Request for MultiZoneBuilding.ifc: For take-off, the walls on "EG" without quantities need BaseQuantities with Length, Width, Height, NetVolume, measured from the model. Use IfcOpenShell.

First a look at what the model holds.

```python
import ifcopenshell
import ifcopenshell.util.element
import ifcopenshell.util.unit

model = ifcopenshell.open("MultiZoneBuilding.ifc")
print(model.schema)
for unit_type in ("LENGTHUNIT", "AREAUNIT", "VOLUMEUNIT"):
    print(unit_type, ifcopenshell.util.unit.calculate_unit_scale(model, unit_type))
storey = next(s for s in model.by_type("IfcBuildingStorey") if s.Name == "EG")
walls = [e for e in ifcopenshell.util.element.get_decomposition(storey) if e.is_a("IfcWall")]
for e in sorted(walls, key=lambda e: e.id()):
    print(e.id(), e.is_a(), e.Name, list(ifcopenshell.util.element.get_psets(e, qtos_only=True)), sep=" | ")
```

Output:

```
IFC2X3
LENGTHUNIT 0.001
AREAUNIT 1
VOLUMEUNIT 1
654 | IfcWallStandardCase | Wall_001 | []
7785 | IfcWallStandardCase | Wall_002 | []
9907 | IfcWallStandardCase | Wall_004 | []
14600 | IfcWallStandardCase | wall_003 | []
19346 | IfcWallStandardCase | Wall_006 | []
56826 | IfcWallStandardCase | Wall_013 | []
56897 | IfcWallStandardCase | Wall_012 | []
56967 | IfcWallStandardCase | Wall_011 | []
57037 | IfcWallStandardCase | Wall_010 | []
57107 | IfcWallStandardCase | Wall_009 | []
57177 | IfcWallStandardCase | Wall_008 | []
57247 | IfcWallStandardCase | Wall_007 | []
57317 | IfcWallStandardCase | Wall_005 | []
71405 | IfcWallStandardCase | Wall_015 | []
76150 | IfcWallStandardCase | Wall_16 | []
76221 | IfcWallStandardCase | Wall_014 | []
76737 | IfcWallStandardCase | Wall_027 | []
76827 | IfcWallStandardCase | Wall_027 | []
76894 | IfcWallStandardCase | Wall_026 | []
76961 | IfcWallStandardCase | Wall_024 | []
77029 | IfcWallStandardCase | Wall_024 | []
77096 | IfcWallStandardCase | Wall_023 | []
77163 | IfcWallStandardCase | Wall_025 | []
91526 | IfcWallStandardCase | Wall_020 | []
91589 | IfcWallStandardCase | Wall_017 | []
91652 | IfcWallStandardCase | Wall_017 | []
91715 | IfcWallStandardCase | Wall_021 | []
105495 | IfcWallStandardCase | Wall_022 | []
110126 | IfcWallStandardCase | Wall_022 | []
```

```python
import ifcopenshell
import ifcopenshell.api.pset
import ifcopenshell.geom
import ifcopenshell.util.element
import ifcopenshell.util.shape
import ifcopenshell.util.unit

model = ifcopenshell.open("MultiZoneBuilding.ifc")
unit_scale = ifcopenshell.util.unit.calculate_unit_scale(model)
volume_scale = ifcopenshell.util.unit.calculate_unit_scale(model, "VOLUMEUNIT")
settings = ifcopenshell.geom.settings()

storey = next(s for s in model.by_type("IfcBuildingStorey") if s.Name == "EG")
walls = [e for e in ifcopenshell.util.element.get_decomposition(storey) if e.is_a("IfcWall")]

for e in sorted(walls, key=lambda e: e.id()):
    if ifcopenshell.util.element.get_psets(e, qtos_only=True, should_inherit=False):
        continue
    # Geometry comes back in metres, in the element's own axes.
    shape = ifcopenshell.geom.create_shape(settings, e)
    values = {
        "Length": ifcopenshell.util.shape.get_x(shape.geometry) / unit_scale,
        "Width": ifcopenshell.util.shape.get_y(shape.geometry) / unit_scale,
        "Height": ifcopenshell.util.shape.get_z(shape.geometry) / unit_scale,
        "NetVolume": ifcopenshell.util.shape.get_volume(shape.geometry) / volume_scale,
    }
    qto = ifcopenshell.api.pset.add_qto(model, product=e, name="BaseQuantities")
    ifcopenshell.api.pset.edit_qto(model, qto=qto, properties=values)
    print(e.id(), {k: round(v, 3) for k, v in values.items()})

model.write("MultiZoneBuilding_rev.ifc")
```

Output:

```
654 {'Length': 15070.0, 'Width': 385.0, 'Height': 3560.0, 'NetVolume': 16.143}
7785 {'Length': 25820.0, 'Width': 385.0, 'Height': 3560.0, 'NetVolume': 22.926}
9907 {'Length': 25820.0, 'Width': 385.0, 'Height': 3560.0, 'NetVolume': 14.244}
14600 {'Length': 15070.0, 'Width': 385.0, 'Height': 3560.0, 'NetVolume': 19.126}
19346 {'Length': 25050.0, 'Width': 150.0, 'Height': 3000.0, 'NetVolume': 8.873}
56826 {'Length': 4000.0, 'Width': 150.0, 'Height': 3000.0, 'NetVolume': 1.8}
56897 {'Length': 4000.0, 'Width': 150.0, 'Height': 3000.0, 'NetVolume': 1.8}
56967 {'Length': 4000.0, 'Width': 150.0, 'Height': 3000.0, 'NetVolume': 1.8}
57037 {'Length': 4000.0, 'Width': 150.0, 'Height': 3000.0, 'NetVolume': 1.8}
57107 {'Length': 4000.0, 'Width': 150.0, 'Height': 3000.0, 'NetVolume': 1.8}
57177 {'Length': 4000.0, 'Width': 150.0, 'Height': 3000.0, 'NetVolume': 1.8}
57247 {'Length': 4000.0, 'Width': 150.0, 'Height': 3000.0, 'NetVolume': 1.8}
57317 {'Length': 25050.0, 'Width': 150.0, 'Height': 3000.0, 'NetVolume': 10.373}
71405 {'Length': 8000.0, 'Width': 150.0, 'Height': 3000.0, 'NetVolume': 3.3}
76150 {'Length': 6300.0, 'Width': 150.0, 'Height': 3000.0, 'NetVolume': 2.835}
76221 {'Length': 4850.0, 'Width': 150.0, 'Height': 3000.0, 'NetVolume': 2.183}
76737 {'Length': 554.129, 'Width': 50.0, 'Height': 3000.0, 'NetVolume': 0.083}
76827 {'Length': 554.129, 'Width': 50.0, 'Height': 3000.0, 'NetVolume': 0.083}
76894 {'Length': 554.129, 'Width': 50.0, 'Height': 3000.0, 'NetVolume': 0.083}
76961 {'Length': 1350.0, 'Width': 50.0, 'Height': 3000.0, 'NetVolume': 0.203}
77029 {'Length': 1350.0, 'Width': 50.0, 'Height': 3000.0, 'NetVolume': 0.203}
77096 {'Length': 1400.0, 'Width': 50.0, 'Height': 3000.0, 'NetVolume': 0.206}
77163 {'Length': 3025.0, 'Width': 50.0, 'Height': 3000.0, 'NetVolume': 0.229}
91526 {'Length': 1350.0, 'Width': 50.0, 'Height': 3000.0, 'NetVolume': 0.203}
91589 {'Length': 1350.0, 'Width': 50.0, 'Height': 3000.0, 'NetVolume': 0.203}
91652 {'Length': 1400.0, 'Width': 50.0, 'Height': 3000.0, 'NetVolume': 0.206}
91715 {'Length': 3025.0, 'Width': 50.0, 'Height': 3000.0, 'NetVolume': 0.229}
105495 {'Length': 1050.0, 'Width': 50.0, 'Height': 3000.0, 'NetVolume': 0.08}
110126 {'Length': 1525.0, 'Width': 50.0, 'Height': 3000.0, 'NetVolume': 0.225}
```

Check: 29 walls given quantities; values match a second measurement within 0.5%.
